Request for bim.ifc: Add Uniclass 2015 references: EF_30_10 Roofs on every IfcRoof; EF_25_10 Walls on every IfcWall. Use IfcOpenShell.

First a look at what the model holds.

```python
import ifcopenshell

model = ifcopenshell.open("bim.ifc")
print(model.schema)
print("classifications:", [c.Name for c in model.by_type("IfcClassification")])
for ifc_class in ("IfcDoor", "IfcRoof", "IfcStair", "IfcWall", "IfcWindow"):
    print(ifc_class, len(model.by_type(ifc_class)))
```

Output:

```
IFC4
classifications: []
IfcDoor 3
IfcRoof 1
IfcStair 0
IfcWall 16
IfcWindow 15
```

```python
import ifcopenshell
import ifcopenshell.api.classification

model = ifcopenshell.open("bim.ifc")

system = ifcopenshell.api.classification.add_classification(model, classification="Uniclass 2015")

codes = {
    "IfcRoof": ("EF_30_10", "Roofs"),
    "IfcWall": ("EF_25_10", "Walls"),
}
for ifc_class, (code, name) in codes.items():
    products = model.by_type(ifc_class)
    ifcopenshell.api.classification.add_reference(
        model, products=products, classification=system, identification=code, name=name
    )
    print(code, len(products))

model.write("bim_v2.ifc")
```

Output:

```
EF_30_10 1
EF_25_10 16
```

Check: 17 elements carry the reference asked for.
